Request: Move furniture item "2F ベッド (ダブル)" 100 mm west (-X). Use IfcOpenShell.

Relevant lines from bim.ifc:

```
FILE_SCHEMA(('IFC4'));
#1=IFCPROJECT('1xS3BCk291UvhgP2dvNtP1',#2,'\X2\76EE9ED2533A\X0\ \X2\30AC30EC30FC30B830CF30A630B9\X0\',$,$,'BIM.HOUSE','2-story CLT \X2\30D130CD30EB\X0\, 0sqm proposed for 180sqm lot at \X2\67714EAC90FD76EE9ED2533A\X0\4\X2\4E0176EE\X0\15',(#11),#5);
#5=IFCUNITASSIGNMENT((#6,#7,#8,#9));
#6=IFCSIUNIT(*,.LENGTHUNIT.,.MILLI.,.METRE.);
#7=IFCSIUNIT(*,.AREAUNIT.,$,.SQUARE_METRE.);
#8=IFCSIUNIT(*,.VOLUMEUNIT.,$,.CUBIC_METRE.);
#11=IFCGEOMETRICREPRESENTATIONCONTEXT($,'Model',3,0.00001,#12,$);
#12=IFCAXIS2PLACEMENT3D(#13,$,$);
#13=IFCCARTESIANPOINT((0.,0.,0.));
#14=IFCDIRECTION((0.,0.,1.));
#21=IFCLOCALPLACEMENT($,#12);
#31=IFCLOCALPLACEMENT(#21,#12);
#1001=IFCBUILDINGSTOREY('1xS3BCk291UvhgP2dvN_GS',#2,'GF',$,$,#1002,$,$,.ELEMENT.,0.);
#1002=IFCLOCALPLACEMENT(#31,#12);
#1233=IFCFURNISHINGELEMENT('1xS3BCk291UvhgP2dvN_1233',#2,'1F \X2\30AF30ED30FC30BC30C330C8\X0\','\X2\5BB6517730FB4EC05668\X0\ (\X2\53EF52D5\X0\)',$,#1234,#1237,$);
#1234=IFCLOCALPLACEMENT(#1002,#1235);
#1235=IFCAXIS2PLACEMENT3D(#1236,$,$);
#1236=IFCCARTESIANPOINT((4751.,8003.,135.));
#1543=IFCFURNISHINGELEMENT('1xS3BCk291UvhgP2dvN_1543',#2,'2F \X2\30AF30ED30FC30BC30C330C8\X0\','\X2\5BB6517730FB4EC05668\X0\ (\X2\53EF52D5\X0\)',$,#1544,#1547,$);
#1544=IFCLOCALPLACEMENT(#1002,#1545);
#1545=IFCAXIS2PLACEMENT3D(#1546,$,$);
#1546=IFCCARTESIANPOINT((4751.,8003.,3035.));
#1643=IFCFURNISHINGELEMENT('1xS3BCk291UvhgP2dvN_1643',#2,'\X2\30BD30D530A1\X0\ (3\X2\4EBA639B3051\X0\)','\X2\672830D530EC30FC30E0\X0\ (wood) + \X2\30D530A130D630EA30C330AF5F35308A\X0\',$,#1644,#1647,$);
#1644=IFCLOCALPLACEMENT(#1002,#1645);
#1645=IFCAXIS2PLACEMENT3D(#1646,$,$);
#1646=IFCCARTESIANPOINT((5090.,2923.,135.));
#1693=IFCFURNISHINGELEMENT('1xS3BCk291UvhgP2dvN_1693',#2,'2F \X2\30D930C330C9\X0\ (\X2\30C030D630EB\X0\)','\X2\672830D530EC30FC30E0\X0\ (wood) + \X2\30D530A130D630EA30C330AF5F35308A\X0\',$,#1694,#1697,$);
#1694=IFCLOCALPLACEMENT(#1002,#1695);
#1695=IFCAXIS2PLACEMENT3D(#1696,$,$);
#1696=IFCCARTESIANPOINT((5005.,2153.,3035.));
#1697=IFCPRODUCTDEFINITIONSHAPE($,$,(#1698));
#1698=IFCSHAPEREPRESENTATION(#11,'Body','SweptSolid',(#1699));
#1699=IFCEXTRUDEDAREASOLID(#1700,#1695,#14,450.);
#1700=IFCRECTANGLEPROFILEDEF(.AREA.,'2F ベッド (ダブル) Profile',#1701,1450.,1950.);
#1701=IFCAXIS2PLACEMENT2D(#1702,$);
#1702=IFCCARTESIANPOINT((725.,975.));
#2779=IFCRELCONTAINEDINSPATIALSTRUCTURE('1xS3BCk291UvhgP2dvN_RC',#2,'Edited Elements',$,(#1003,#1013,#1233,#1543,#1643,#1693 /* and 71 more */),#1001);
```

```python
import ifcopenshell
import ifcopenshell.api.geometry
import ifcopenshell.util.placement

model = ifcopenshell.open("bim.ifc")

item = model.by_guid("1xS3BCk291UvhgP2dvN_1693")
matrix = ifcopenshell.util.placement.get_local_placement(item.ObjectPlacement)
matrix[0, 3] -= 100.0
ifcopenshell.api.geometry.edit_object_placement(model, product=item, matrix=matrix, is_si=False)

print(ifcopenshell.util.placement.get_local_placement(item.ObjectPlacement).round(3) + 0.0)

model.write("bim_v2.ifc")
```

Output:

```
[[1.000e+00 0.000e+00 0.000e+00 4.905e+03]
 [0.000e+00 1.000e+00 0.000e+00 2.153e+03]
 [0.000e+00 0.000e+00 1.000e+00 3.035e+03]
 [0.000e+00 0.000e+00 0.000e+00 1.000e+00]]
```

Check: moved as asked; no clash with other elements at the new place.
